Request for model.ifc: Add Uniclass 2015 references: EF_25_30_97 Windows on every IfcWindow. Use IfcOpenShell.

First a look at what the model holds.

```python
import ifcopenshell

model = ifcopenshell.open("model.ifc")
print(model.schema)
print("classifications:", [c.Name for c in model.by_type("IfcClassification")])
for ifc_class in ("IfcDoor", "IfcRoof", "IfcStair", "IfcWall", "IfcWindow"):
    print(ifc_class, len(model.by_type(ifc_class)))
```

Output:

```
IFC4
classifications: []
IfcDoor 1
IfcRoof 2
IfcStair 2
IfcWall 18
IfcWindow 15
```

```python
import ifcopenshell
import ifcopenshell.api.classification

model = ifcopenshell.open("model.ifc")

system = ifcopenshell.api.classification.add_classification(model, classification="Uniclass 2015")

codes = {
    "IfcWindow": ("EF_25_30_97", "Windows"),
}
for ifc_class, (code, name) in codes.items():
    products = model.by_type(ifc_class)
    ifcopenshell.api.classification.add_reference(
        model, products=products, classification=system, identification=code, name=name
    )
    print(code, len(products))

model.write("model_edited.ifc")
```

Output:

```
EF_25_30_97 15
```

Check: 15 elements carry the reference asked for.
